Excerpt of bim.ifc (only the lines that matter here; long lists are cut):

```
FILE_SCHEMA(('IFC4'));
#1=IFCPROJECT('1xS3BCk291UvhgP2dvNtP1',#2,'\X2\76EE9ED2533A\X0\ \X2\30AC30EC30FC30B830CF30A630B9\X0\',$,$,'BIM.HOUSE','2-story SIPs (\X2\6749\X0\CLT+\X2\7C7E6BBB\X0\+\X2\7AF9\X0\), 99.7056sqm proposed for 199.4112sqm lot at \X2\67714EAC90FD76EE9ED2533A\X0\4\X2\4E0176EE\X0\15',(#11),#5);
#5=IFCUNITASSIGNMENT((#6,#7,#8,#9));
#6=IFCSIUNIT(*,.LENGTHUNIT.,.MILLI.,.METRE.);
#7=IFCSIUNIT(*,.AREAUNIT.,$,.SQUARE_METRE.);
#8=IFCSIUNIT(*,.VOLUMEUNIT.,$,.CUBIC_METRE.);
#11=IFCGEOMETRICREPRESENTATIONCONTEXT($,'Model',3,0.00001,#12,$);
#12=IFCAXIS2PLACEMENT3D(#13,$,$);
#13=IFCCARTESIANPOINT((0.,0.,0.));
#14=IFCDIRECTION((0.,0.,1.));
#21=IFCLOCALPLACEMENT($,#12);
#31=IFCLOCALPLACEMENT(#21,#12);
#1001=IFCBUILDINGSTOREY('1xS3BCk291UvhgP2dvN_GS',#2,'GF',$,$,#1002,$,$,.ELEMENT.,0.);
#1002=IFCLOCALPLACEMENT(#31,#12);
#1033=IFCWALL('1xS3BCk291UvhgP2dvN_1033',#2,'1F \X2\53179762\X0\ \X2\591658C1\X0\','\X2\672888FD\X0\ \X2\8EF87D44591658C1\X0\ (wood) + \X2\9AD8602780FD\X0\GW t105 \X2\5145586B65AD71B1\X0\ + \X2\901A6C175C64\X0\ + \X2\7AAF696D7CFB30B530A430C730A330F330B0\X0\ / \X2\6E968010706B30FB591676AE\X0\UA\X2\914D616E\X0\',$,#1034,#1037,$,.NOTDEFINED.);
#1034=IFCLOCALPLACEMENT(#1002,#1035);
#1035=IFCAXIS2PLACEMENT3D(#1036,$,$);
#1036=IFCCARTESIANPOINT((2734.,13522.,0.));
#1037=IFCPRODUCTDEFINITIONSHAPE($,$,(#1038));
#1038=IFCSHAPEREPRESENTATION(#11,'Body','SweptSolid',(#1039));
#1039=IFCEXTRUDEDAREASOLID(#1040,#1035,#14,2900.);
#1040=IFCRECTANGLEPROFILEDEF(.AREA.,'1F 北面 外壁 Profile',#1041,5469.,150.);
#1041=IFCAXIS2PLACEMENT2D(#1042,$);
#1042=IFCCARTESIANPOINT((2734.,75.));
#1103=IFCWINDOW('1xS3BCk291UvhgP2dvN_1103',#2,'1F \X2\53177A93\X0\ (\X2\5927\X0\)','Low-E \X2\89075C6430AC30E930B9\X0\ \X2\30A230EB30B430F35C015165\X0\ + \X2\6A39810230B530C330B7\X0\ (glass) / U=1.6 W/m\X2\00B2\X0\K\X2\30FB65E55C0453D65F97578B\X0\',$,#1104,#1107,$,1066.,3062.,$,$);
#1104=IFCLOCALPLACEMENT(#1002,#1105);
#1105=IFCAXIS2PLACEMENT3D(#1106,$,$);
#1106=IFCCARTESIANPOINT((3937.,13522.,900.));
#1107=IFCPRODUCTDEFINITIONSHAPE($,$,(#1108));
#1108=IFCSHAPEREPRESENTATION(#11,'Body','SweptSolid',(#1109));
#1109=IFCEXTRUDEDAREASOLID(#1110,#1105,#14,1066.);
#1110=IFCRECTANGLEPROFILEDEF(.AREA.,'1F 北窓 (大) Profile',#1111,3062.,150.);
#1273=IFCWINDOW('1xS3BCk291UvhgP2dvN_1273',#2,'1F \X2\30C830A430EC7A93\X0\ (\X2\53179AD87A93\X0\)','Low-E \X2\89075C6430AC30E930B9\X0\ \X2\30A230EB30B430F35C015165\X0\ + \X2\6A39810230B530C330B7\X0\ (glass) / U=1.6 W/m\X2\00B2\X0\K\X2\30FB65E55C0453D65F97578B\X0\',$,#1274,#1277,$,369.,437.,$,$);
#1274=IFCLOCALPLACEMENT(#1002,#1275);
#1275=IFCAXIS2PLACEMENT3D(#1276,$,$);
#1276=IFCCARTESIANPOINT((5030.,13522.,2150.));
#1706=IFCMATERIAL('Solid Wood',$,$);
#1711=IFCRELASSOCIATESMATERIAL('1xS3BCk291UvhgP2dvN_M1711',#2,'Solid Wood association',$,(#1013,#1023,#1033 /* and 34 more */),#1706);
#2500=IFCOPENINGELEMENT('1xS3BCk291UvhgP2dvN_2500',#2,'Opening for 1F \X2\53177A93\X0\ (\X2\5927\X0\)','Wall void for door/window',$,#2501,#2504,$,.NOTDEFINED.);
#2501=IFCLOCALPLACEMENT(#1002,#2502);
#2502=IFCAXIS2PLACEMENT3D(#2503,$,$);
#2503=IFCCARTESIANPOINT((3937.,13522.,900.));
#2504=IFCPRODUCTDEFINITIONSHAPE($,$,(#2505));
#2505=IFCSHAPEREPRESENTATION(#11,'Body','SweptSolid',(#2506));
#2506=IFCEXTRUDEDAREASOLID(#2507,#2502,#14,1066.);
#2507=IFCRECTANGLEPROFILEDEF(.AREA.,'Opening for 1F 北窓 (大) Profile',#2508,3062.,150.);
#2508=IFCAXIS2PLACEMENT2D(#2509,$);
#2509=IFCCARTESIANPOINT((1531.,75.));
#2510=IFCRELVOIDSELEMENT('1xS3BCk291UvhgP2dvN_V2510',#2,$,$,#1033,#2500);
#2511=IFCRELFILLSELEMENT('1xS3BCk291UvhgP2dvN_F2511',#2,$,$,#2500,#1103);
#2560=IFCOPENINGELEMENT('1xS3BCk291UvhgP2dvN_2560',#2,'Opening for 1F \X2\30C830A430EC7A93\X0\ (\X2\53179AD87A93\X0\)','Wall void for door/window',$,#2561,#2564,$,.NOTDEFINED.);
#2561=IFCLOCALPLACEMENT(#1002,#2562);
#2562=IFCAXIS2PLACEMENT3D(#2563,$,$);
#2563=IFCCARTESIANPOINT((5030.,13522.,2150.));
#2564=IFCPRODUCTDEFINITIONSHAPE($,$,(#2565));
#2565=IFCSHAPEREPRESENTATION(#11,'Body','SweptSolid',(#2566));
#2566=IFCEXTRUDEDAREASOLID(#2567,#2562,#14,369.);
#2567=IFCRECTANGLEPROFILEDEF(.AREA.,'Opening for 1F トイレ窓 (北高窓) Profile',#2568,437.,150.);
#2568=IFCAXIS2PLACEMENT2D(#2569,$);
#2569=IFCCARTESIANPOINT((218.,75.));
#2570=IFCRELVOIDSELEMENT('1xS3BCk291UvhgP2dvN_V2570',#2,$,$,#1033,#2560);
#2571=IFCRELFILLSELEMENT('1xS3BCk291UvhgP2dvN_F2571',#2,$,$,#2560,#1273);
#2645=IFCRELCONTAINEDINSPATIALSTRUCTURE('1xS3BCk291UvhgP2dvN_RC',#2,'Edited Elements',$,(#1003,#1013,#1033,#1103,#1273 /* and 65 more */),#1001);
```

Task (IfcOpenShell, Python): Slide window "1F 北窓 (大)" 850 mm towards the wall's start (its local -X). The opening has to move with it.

```python
import ifcopenshell
import ifcopenshell.api.geometry
import ifcopenshell.util.placement

model = ifcopenshell.open("bim.ifc")

window = model.by_guid("1xS3BCk291UvhgP2dvN_1103")
opening = window.FillsVoids[0].RelatingOpeningElement
wall = opening.VoidsElements[0].RelatingBuildingElement

wall_matrix = ifcopenshell.util.placement.get_local_placement(wall.ObjectPlacement)
shift = wall_matrix[:3, 0] * -850.0
before = ifcopenshell.util.placement.get_local_placement(window.ObjectPlacement)[:3, 3].copy()

# The window is not placed relative to its opening, so move both.
for product in (opening, window):
    matrix = ifcopenshell.util.placement.get_local_placement(product.ObjectPlacement)
    matrix[:3, 3] += shift
    ifcopenshell.api.geometry.edit_object_placement(model, product=product, matrix=matrix, is_si=False)

after = ifcopenshell.util.placement.get_local_placement(window.ObjectPlacement)[:3, 3]
print("window moved by", (after - before).round(3) + 0.0)

model.write("bim_edited.ifc")
```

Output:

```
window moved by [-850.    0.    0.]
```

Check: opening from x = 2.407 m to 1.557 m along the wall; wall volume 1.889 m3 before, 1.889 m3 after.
